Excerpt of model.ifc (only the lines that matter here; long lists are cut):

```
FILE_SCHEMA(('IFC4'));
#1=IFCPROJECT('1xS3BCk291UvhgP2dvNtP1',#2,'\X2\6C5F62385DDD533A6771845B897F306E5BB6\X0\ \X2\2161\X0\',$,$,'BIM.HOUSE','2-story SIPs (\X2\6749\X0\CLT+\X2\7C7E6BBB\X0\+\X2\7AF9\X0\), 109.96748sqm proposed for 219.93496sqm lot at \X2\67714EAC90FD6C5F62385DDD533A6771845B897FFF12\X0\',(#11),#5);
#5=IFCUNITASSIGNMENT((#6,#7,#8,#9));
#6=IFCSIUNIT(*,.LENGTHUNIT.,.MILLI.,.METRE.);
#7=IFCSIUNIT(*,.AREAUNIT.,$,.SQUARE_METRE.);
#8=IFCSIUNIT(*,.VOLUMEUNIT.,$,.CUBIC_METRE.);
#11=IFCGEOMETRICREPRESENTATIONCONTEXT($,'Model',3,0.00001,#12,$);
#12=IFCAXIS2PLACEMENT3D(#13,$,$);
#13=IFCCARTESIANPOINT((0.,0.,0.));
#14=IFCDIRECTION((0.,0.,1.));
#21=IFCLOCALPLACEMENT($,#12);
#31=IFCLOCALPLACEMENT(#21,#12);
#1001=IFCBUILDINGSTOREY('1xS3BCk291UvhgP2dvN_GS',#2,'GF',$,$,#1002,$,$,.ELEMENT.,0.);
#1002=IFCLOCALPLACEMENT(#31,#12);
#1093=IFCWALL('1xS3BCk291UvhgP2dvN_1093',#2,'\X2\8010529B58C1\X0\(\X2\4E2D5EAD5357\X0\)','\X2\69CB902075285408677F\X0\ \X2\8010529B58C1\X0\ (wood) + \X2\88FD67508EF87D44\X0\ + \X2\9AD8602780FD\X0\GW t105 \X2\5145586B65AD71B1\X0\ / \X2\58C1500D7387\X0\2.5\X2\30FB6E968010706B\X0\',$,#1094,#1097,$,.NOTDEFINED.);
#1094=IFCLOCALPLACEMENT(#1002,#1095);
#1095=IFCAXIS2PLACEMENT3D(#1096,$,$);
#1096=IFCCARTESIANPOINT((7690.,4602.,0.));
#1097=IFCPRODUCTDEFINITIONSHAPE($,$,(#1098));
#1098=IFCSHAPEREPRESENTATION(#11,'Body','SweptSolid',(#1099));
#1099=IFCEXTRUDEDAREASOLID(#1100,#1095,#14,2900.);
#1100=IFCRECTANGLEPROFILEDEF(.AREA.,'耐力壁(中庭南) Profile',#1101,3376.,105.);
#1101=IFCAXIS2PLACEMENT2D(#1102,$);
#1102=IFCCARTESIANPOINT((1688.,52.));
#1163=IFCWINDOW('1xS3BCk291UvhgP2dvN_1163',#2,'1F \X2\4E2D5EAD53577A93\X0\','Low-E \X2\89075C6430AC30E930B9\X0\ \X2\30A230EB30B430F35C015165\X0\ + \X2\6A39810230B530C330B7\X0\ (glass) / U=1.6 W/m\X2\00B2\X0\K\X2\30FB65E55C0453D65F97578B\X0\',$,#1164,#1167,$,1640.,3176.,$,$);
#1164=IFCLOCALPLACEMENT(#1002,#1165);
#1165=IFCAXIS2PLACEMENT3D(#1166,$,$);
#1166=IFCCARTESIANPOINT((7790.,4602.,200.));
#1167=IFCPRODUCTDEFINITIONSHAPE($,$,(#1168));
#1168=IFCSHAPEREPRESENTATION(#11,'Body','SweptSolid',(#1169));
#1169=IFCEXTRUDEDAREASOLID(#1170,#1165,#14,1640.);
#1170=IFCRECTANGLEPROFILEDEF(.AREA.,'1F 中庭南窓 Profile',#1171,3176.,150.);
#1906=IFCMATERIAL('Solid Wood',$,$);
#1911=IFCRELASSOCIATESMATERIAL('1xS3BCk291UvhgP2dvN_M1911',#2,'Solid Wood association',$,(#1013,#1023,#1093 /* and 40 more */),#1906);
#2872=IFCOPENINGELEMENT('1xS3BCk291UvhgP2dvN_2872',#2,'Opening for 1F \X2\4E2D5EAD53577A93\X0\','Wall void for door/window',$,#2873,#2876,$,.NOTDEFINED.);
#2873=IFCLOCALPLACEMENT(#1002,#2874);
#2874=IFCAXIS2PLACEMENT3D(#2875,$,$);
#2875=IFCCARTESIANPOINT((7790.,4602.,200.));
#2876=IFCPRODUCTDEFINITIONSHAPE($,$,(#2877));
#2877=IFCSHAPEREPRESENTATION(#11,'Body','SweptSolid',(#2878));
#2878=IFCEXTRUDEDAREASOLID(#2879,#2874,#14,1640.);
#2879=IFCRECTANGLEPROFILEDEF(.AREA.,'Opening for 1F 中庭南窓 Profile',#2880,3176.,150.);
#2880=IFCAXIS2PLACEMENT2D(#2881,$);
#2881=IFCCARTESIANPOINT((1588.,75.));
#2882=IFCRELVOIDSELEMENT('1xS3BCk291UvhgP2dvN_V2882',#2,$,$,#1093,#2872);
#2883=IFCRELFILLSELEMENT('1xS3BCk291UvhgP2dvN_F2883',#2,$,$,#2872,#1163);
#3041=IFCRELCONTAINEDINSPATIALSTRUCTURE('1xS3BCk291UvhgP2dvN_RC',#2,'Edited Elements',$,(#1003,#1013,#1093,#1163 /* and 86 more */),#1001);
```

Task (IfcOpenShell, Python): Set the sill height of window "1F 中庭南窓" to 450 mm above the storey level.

```python
import numpy as np
import ifcopenshell
import ifcopenshell.api.geometry
import ifcopenshell.geom
import ifcopenshell.util.element
import ifcopenshell.util.placement
import ifcopenshell.util.shape
import ifcopenshell.util.unit

model = ifcopenshell.open("model.ifc")
unit_scale = ifcopenshell.util.unit.calculate_unit_scale(model)

window = model.by_guid("1xS3BCk291UvhgP2dvN_1163")
opening = window.FillsVoids[0].RelatingOpeningElement
storey = ifcopenshell.util.element.get_container(window, ifc_class="IfcBuildingStorey")
level = ifcopenshell.util.placement.get_local_placement(storey.ObjectPlacement)[2, 3]

# The opening's origin need not be at the sill, so measure its lowest point.
shape = ifcopenshell.geom.create_shape(ifcopenshell.geom.settings(), opening)
bottom = ifcopenshell.util.shape.get_shape_bottom_elevation(shape, shape.geometry) / unit_scale
dz = level + 0.45 / unit_scale - bottom

shift = np.array([0.0, 0.0, dz])
# The window is not placed relative to its opening, so move both.
for product in (opening, window):
    matrix = ifcopenshell.util.placement.get_local_placement(product.ObjectPlacement)
    matrix[:3, 3] += shift
    ifcopenshell.api.geometry.edit_object_placement(model, product=product, matrix=matrix, is_si=False)

print(f"moved by {dz * unit_scale:+.3f} m")

model.write("model-out.ifc")
```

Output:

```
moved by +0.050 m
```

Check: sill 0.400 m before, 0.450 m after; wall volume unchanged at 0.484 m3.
